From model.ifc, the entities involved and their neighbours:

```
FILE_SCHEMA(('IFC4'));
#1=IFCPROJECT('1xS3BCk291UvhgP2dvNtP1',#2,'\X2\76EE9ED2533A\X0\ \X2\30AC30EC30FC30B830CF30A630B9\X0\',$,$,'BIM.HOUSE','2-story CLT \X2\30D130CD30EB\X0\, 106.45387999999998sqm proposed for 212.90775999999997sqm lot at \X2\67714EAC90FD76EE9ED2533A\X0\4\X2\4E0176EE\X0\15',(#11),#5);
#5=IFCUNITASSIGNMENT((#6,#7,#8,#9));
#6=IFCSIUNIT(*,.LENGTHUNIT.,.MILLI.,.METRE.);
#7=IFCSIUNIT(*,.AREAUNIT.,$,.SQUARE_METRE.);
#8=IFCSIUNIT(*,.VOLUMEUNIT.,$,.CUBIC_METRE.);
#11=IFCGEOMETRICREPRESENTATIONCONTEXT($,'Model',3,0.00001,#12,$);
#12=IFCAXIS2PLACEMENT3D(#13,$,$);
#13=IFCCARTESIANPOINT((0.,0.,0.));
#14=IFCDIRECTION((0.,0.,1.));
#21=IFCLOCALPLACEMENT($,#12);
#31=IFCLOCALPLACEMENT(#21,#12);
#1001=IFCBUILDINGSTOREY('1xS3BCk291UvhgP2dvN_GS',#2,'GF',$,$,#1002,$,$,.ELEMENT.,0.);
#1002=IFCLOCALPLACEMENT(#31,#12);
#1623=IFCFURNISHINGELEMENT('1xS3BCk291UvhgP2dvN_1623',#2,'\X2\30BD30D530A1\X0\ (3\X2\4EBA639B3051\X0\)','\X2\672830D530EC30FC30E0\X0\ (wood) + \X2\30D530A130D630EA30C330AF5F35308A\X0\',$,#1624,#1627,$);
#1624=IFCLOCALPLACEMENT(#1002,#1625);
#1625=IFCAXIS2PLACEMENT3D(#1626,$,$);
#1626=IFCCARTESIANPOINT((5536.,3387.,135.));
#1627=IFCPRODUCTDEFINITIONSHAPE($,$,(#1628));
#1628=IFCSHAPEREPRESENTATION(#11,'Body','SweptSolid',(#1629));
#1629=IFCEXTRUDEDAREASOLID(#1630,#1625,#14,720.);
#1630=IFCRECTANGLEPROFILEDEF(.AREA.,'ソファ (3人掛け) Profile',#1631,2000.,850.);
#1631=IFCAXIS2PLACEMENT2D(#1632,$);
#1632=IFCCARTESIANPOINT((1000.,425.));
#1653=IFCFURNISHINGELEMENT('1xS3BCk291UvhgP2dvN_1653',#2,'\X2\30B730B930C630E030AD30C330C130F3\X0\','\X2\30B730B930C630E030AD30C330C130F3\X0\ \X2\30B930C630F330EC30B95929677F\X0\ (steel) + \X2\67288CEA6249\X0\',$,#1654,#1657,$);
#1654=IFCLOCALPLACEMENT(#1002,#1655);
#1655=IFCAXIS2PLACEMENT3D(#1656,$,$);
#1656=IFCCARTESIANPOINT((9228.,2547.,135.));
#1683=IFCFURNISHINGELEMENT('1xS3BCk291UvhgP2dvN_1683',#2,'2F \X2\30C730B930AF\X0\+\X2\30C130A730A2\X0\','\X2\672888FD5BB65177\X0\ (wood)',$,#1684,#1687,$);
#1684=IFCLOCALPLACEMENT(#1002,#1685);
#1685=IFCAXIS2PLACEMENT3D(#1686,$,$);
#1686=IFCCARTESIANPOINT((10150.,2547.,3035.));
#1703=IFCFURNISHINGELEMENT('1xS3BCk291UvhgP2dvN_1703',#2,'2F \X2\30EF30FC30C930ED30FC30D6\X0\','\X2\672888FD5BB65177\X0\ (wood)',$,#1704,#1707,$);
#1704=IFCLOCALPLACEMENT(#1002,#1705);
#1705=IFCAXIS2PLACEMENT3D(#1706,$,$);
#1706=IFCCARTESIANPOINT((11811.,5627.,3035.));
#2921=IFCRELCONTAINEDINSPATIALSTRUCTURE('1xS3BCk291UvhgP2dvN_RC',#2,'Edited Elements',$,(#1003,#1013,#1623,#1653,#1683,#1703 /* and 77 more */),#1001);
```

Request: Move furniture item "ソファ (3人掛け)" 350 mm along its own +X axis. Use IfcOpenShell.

```python
import ifcopenshell
import ifcopenshell.api.geometry
import ifcopenshell.util.placement

model = ifcopenshell.open("model.ifc")

item = model.by_guid("1xS3BCk291UvhgP2dvN_1623")
matrix = ifcopenshell.util.placement.get_local_placement(item.ObjectPlacement)
matrix[:3, 3] += matrix[:3, 0] * 350.0
ifcopenshell.api.geometry.edit_object_placement(model, product=item, matrix=matrix, is_si=False)

print(ifcopenshell.util.placement.get_local_placement(item.ObjectPlacement).round(3) + 0.0)

model.write("model_updated.ifc")
```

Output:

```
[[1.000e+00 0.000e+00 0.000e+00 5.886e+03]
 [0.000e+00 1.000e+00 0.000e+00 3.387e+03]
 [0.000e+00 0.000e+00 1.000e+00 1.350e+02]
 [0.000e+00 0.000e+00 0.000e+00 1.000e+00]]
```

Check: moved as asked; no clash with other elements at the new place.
